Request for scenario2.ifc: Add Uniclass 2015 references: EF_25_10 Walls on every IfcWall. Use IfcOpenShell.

First a look at what the model holds.

```python
import ifcopenshell

model = ifcopenshell.open("scenario2.ifc")
print(model.schema)
print("classifications:", [c.Name for c in model.by_type("IfcClassification")])
for ifc_class in ("IfcDoor", "IfcRoof", "IfcStair", "IfcWall", "IfcWindow"):
    print(ifc_class, len(model.by_type(ifc_class)))
```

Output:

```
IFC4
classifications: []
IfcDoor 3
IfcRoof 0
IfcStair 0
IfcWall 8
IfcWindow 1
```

```python
import ifcopenshell
import ifcopenshell.api.classification

model = ifcopenshell.open("scenario2.ifc")

system = ifcopenshell.api.classification.add_classification(model, classification="Uniclass 2015")

codes = {
    "IfcWall": ("EF_25_10", "Walls"),
}
for ifc_class, (code, name) in codes.items():
    products = model.by_type(ifc_class)
    ifcopenshell.api.classification.add_reference(
        model, products=products, classification=system, identification=code, name=name
    )
    print(code, len(products))

model.write("scenario2_edited.ifc")
```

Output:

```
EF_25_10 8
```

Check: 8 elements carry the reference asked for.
